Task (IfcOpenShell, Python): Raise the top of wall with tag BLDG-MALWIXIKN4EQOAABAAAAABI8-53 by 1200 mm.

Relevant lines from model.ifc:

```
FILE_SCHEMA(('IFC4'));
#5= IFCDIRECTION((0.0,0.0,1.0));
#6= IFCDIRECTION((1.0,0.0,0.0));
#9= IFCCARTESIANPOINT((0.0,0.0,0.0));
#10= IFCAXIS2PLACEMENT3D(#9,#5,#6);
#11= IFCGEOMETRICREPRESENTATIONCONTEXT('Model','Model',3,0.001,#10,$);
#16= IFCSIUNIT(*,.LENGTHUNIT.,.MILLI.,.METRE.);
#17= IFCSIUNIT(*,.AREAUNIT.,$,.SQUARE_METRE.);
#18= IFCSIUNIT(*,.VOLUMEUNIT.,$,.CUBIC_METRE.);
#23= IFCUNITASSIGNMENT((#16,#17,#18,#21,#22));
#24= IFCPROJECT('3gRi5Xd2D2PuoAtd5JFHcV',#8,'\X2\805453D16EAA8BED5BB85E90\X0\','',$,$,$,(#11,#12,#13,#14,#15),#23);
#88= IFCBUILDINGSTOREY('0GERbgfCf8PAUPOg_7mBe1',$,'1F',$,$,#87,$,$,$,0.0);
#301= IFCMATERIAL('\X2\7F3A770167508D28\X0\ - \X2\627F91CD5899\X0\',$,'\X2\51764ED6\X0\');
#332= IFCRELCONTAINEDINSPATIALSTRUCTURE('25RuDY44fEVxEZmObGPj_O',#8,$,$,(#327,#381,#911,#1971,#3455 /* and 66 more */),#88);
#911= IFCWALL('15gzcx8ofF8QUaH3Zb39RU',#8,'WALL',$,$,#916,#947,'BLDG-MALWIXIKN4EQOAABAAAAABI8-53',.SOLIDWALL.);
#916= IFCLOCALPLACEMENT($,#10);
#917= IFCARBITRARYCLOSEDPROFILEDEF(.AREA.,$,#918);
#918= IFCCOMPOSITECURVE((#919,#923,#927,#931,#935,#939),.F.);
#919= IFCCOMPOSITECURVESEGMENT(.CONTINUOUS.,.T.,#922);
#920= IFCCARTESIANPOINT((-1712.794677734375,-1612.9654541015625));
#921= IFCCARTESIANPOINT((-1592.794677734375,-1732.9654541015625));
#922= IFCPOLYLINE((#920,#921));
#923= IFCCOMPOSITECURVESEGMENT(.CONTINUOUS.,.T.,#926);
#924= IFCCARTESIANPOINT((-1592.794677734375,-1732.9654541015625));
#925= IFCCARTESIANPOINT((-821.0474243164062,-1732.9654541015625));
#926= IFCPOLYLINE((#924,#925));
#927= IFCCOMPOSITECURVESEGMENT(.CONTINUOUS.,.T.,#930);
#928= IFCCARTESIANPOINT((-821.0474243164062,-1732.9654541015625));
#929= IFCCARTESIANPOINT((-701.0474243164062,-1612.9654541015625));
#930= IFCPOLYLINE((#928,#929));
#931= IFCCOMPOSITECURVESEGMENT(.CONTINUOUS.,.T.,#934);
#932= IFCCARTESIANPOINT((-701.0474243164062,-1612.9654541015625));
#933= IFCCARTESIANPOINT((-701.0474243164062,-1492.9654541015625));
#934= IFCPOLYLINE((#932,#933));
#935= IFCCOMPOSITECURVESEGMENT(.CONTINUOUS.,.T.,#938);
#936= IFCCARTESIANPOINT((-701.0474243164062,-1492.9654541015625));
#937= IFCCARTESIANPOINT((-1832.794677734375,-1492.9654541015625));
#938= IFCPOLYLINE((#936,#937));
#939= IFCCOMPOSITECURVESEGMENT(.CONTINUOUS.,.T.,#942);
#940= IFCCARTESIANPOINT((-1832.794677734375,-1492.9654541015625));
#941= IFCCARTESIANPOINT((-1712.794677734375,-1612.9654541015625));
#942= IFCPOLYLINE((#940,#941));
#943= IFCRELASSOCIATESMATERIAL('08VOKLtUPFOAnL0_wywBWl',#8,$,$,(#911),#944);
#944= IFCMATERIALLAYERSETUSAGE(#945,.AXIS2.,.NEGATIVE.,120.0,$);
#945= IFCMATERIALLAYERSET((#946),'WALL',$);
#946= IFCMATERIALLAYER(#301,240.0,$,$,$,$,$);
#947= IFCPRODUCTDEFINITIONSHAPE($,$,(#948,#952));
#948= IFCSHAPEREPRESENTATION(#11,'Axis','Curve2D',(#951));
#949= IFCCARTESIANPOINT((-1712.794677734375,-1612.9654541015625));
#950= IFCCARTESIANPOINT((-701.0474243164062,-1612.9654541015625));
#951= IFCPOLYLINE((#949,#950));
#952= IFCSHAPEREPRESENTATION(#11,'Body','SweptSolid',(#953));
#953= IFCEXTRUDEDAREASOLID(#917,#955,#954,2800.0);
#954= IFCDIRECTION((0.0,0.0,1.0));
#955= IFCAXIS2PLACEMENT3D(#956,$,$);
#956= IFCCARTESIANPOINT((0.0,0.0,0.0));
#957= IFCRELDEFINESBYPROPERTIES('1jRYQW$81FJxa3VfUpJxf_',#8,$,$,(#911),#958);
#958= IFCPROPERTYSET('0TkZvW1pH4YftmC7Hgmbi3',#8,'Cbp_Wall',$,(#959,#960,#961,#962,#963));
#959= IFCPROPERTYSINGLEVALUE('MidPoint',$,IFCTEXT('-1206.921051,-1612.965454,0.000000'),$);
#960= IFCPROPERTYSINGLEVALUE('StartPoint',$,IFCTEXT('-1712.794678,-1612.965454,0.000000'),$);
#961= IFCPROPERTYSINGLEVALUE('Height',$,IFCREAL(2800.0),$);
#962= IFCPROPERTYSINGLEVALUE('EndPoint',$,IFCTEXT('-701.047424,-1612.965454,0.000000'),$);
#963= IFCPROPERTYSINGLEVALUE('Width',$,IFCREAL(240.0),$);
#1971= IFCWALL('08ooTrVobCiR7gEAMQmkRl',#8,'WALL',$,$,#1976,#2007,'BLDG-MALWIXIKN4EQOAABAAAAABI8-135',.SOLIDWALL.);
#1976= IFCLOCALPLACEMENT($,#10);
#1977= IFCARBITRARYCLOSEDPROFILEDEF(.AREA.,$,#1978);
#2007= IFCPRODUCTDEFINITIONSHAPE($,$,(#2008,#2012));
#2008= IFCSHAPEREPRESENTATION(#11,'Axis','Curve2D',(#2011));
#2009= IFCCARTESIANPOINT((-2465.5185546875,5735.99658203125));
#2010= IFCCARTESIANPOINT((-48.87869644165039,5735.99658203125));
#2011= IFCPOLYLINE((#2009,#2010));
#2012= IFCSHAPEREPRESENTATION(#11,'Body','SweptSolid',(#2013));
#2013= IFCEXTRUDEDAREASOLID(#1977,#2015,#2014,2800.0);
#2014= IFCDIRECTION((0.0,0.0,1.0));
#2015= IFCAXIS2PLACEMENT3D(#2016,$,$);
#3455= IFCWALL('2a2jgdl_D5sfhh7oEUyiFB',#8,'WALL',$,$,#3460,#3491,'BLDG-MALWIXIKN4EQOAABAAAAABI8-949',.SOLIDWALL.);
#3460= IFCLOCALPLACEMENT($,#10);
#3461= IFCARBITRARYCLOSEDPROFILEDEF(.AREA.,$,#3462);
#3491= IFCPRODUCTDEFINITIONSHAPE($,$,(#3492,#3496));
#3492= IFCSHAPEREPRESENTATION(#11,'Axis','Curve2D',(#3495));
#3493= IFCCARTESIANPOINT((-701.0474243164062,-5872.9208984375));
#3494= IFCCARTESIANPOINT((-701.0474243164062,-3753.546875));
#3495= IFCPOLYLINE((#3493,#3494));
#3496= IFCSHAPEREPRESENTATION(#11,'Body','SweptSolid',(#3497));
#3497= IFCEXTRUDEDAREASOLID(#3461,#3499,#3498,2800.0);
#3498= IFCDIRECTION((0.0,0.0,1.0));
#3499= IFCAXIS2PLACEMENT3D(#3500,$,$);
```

```python
import ifcopenshell
import ifcopenshell.api.pset
import ifcopenshell.geom
import ifcopenshell.util.element
import ifcopenshell.util.shape
import ifcopenshell.util.unit

model = ifcopenshell.open("model.ifc")
unit_scale = ifcopenshell.util.unit.calculate_unit_scale(model)
settings = ifcopenshell.geom.settings()


def volume(element):
    """Net volume in cubic metres, openings subtracted."""
    shape = ifcopenshell.geom.create_shape(settings, element)
    return ifcopenshell.util.shape.get_volume(shape.geometry)


wall = model.by_id(911)
before = volume(wall)

body = next(r for r in wall.Representation.Representations if r.RepresentationIdentifier == "Body")
solid = body.Items[0]
old_height = solid.Depth
solid.Depth += 1.2 / unit_scale
after = volume(wall)

# Update the stored height, areas and volumes.
pset = model.by_id(ifcopenshell.util.element.get_pset(wall, "Cbp_Wall", should_inherit=False)["id"])
ifcopenshell.api.pset.edit_pset(model, pset=pset, properties={"Height": model.create_entity("IfcReal", solid.Depth)})

print(f"height {old_height:g} -> {solid.Depth:g}, volume {before:.3f} -> {after:.3f} m3")

model.write("model_v2.ifc")
```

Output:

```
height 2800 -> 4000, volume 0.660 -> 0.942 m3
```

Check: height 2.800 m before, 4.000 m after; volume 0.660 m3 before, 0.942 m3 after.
